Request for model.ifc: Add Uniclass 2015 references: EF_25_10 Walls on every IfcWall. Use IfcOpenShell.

First a look at what the model holds.

```python
import ifcopenshell

model = ifcopenshell.open("model.ifc")
print(model.schema)
print("classifications:", [c.Name for c in model.by_type("IfcClassification")])
for ifc_class in ("IfcDoor", "IfcRoof", "IfcStair", "IfcWall", "IfcWindow"):
    print(ifc_class, len(model.by_type(ifc_class)))
```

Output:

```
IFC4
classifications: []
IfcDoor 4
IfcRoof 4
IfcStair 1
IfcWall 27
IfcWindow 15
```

```python
import ifcopenshell
import ifcopenshell.api.classification

model = ifcopenshell.open("model.ifc")

system = ifcopenshell.api.classification.add_classification(model, classification="Uniclass 2015")

codes = {
    "IfcWall": ("EF_25_10", "Walls"),
}
for ifc_class, (code, name) in codes.items():
    products = model.by_type(ifc_class)
    ifcopenshell.api.classification.add_reference(
        model, products=products, classification=system, identification=code, name=name
    )
    print(code, len(products))

model.write("model_rev.ifc")
```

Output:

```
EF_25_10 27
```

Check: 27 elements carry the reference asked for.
